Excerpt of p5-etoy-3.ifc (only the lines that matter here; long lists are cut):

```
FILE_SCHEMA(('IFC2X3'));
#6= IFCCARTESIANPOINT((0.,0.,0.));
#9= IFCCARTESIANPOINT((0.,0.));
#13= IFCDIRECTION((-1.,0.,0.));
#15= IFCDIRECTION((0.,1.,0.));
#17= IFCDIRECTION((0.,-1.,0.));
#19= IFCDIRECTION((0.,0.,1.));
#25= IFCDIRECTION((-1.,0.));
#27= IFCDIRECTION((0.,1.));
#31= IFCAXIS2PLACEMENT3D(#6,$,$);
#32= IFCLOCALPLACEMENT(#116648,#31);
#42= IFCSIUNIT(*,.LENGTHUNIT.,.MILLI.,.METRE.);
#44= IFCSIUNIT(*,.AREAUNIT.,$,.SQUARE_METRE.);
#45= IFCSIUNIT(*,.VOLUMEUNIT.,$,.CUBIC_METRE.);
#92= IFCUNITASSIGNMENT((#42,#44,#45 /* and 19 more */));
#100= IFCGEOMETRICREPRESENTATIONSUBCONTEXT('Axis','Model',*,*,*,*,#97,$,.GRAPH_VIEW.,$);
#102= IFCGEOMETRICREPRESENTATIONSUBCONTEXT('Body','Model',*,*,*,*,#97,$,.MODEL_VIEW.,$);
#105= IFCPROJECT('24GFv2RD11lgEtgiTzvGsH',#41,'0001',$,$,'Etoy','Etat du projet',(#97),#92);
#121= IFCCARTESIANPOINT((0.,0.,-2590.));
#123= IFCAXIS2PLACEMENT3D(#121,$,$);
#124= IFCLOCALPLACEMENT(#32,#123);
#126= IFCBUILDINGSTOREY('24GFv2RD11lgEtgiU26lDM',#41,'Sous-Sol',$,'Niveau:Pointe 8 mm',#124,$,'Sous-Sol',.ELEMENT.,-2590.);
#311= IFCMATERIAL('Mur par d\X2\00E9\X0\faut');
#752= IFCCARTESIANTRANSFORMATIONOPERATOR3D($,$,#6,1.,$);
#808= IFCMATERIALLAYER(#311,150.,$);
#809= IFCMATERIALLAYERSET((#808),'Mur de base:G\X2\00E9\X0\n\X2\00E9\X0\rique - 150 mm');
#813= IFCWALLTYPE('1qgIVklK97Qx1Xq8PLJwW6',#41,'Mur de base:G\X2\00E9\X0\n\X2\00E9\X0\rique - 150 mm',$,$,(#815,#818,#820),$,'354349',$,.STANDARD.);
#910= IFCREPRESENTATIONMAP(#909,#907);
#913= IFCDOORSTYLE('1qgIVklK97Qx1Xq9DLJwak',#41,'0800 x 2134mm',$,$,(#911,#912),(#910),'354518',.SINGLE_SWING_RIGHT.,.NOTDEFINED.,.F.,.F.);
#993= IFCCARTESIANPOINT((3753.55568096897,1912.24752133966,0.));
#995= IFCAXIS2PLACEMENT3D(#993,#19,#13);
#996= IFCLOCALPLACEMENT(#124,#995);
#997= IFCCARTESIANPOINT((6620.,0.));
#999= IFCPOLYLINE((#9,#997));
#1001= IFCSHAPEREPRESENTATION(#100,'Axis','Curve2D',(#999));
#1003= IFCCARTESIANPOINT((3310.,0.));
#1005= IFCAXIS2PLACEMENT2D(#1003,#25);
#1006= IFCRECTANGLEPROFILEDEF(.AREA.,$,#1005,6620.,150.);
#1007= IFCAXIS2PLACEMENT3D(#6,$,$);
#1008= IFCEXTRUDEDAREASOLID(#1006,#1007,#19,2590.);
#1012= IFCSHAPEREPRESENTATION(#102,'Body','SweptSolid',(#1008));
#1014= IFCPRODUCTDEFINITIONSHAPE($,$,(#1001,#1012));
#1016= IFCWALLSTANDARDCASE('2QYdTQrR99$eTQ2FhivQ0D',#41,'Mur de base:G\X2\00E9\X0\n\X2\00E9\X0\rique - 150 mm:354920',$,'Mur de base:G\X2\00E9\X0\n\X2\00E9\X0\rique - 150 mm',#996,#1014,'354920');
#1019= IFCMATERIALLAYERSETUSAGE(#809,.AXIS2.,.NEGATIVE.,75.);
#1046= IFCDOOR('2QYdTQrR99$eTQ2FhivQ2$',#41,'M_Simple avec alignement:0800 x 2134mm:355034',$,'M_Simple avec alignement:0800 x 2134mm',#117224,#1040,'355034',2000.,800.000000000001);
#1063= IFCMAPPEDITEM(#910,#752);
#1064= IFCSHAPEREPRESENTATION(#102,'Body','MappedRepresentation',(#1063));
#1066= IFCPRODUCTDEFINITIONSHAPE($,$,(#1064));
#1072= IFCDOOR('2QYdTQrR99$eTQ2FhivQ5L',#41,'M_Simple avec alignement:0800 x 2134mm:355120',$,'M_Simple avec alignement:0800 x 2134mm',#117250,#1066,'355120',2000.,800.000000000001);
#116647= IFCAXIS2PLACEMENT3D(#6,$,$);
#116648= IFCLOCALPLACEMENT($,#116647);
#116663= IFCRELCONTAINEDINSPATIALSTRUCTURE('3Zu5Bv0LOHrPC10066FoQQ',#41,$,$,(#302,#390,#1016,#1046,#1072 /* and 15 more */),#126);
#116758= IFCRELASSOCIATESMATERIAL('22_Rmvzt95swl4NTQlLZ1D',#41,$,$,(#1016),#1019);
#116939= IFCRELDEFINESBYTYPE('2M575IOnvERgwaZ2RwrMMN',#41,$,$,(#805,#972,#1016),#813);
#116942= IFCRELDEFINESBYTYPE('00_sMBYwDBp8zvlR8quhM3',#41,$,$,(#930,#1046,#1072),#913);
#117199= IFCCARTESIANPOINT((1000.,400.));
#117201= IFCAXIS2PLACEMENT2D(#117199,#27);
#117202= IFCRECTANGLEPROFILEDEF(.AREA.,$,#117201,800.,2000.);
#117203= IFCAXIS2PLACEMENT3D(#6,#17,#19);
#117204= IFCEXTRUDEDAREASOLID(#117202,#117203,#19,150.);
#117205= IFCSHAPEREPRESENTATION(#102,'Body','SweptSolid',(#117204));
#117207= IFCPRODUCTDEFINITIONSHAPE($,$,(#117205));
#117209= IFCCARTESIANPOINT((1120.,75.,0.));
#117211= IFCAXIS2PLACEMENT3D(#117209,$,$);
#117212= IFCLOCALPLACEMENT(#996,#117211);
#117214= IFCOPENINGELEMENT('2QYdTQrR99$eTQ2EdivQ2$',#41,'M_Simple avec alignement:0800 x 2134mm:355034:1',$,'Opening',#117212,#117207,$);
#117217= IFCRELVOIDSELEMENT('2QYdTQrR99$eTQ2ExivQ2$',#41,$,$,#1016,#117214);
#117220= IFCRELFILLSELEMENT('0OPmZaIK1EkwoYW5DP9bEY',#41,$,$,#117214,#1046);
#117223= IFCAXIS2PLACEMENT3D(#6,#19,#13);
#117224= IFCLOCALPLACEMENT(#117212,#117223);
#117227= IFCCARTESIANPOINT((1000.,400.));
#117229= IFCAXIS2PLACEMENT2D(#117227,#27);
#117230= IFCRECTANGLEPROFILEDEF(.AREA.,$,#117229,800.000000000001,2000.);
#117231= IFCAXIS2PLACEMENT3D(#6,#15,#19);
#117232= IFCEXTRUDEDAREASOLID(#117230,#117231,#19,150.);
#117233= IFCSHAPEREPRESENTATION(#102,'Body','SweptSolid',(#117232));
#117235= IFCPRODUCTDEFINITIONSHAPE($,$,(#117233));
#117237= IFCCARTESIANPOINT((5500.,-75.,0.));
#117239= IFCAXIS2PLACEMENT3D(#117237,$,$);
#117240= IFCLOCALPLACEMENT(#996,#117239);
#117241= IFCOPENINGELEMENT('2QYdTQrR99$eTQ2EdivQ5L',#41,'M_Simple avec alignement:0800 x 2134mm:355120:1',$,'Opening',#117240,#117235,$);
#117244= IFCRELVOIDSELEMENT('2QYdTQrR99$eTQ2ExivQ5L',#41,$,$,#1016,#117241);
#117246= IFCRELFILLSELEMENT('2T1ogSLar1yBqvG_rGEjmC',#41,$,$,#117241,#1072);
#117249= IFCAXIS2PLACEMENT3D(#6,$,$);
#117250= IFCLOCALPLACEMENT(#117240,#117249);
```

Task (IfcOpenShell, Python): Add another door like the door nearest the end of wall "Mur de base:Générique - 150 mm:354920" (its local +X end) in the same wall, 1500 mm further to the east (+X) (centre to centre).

```python
import ifcopenshell
import ifcopenshell.api.feature
import ifcopenshell.api.geometry
import ifcopenshell.api.root
import ifcopenshell.geom
import ifcopenshell.util.element
import ifcopenshell.util.placement
import ifcopenshell.util.shape
import ifcopenshell.util.unit

model = ifcopenshell.open("p5-etoy-3.ifc")
unit_scale = ifcopenshell.util.unit.calculate_unit_scale(model)
settings = ifcopenshell.geom.settings()


def volume(element):
    """Net volume in cubic metres, openings subtracted."""
    shape = ifcopenshell.geom.create_shape(settings, element)
    return ifcopenshell.util.shape.get_volume(shape.geometry)


def reuse_history(source, copy):
    """copy_class also copies each property set's owner history, people and application; keep the originals."""
    for rel in copy.IsDefinedBy:
        if rel.is_a("IfcRelDefinesByProperties") and (history := rel.RelatingPropertyDefinition.OwnerHistory):
            rel.RelatingPropertyDefinition.OwnerHistory = source.OwnerHistory
            ifcopenshell.util.element.remove_deep2(model, history)


door = model.by_id(1072)
opening = door.FillsVoids[0].RelatingOpeningElement
wall = opening.VoidsElements[0].RelatingBuildingElement
before = volume(wall)
shift = ifcopenshell.util.placement.get_local_placement(wall.ObjectPlacement)[:3, 0] * -1.5 / unit_scale

# copy_class copies the void relationship, type, container and properties, but no geometry.
new_opening = ifcopenshell.api.root.copy_class(model, product=opening)
new_opening.Representation = ifcopenshell.util.element.copy_deep(
    model, opening.Representation, exclude=["IfcGeometricRepresentationContext", "IfcRepresentationMap"]
)
new_opening.Name = "M_Simple avec alignement:0800 x 2134mm"
new_door = ifcopenshell.api.root.copy_class(model, product=door)
new_door.Representation = ifcopenshell.util.element.copy_deep(
    model, door.Representation, exclude=["IfcGeometricRepresentationContext", "IfcRepresentationMap"]
)
new_door.Name = "M_Simple avec alignement:0800 x 2134mm"
new_door.Tag = None
reuse_history(door, new_door)
fills = ifcopenshell.api.feature.add_filling(model, opening=new_opening, element=new_door)
fills.OwnerHistory = new_door.OwnerHistory  # required in IFC2X3

for old, new in ((opening, new_opening), (door, new_door)):
    matrix = ifcopenshell.util.placement.get_local_placement(old.ObjectPlacement)
    matrix[:3, 3] += shift
    ifcopenshell.api.geometry.edit_object_placement(model, product=new, matrix=matrix, is_si=False)

after = volume(wall)

print(f"wall volume {before:.3f} -> {after:.3f} m3")

model.write("p5-etoy-3-out.ifc")
```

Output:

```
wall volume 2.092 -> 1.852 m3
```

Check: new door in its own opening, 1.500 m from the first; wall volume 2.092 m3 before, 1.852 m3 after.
